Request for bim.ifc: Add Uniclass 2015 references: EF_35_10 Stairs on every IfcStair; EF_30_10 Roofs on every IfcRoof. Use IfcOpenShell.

First a look at what the model holds.

```python
import ifcopenshell

model = ifcopenshell.open("bim.ifc")
print(model.schema)
print("classifications:", [c.Name for c in model.by_type("IfcClassification")])
for ifc_class in ("IfcDoor", "IfcRoof", "IfcStair", "IfcWall", "IfcWindow"):
    print(ifc_class, len(model.by_type(ifc_class)))
```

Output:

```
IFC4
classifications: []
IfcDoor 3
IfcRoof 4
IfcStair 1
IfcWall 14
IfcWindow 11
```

```python
import ifcopenshell
import ifcopenshell.api.classification

model = ifcopenshell.open("bim.ifc")

system = ifcopenshell.api.classification.add_classification(model, classification="Uniclass 2015")

codes = {
    "IfcStair": ("EF_35_10", "Stairs"),
    "IfcRoof": ("EF_30_10", "Roofs"),
}
for ifc_class, (code, name) in codes.items():
    products = model.by_type(ifc_class)
    ifcopenshell.api.classification.add_reference(
        model, products=products, classification=system, identification=code, name=name
    )
    print(code, len(products))

model.write("bim_edited.ifc")
```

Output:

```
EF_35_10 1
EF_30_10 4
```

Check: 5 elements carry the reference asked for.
